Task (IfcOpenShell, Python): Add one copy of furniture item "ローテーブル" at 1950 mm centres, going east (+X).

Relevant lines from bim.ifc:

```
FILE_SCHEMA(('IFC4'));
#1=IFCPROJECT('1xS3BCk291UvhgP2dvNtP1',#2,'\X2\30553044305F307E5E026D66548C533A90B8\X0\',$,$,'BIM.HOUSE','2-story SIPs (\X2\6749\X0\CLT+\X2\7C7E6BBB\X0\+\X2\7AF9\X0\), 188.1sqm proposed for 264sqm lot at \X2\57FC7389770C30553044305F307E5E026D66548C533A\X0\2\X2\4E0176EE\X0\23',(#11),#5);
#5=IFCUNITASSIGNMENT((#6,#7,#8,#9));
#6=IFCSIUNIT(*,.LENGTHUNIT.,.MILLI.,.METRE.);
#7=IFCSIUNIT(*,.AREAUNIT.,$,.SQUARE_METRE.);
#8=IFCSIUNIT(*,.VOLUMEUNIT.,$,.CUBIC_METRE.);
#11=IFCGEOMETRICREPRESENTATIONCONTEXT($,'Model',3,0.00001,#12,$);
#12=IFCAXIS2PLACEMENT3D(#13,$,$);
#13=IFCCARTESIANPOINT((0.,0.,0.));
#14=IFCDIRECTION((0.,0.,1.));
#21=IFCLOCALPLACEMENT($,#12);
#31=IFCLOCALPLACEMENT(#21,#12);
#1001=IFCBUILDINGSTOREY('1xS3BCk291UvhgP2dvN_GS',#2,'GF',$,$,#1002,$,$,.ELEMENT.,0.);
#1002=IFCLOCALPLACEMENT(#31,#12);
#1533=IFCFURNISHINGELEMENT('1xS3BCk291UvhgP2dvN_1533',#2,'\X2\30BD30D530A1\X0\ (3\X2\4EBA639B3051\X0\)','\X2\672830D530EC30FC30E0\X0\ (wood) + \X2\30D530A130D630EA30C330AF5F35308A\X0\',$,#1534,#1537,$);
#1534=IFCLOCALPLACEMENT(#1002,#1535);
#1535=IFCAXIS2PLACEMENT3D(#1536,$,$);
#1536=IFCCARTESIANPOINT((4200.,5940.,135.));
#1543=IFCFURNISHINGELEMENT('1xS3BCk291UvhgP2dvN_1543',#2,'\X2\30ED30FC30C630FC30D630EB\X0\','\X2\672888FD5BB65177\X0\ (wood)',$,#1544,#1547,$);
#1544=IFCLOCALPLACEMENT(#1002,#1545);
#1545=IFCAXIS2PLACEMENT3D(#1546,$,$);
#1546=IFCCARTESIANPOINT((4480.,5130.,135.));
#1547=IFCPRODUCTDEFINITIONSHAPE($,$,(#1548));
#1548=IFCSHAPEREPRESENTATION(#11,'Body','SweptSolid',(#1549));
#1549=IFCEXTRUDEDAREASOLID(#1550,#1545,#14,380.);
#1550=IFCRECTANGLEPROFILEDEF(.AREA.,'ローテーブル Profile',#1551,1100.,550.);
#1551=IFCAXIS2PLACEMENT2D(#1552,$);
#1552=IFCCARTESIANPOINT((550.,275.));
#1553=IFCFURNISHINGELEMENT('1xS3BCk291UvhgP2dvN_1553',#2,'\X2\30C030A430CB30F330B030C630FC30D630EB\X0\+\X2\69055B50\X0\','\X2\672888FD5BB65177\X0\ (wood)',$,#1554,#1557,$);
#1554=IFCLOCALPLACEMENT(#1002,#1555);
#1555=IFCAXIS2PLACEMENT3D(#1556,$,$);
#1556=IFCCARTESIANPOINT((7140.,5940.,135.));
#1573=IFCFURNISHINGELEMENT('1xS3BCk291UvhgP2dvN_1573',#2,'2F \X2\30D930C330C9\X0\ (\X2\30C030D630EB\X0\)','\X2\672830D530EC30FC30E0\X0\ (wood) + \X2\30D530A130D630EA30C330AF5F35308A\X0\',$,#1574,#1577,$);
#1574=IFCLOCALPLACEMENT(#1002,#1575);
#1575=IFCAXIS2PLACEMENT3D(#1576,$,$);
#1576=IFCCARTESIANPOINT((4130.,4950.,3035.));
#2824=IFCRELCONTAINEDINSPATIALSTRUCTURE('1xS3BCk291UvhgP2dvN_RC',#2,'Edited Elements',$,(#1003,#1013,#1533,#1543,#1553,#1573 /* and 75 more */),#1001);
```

```python
import numpy as np
import ifcopenshell
import ifcopenshell.api.geometry
import ifcopenshell.api.root
import ifcopenshell.util.element
import ifcopenshell.util.placement

model = ifcopenshell.open("bim.ifc")


def reuse_history(source, copy):
    """copy_class also copies each property set's owner history, people and application; keep the originals."""
    for rel in copy.IsDefinedBy:
        if rel.is_a("IfcRelDefinesByProperties") and (history := rel.RelatingPropertyDefinition.OwnerHistory):
            rel.RelatingPropertyDefinition.OwnerHistory = source.OwnerHistory
            ifcopenshell.util.element.remove_deep2(model, history)


source = model.by_id(1543)
base = ifcopenshell.util.placement.get_local_placement(source.ObjectPlacement)
step = np.array([1.0, 0.0, 0.0]) * 1950.0

for i in range(1, 2):
    copy = ifcopenshell.api.root.copy_class(model, product=source)
    copy.Representation = ifcopenshell.util.element.copy_deep(
        model, source.Representation, exclude=["IfcGeometricRepresentationContext", "IfcRepresentationMap"]
    )
    reuse_history(source, copy)
    matrix = base.copy()
    matrix[:3, 3] += i * step
    print("added at", matrix[:3, 3].round(3) + 0.0)
    ifcopenshell.api.geometry.edit_object_placement(model, product=copy, matrix=matrix, is_si=False)

model.write("bim_updated.ifc")
```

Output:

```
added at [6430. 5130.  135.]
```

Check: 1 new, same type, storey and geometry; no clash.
